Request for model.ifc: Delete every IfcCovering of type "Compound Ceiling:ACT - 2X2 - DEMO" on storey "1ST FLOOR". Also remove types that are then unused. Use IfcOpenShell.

First a look at what the model holds.

```python
import ifcopenshell
import ifcopenshell.util.element

model = ifcopenshell.open("model.ifc")
print(model.schema)
storey = next(s for s in model.by_type("IfcBuildingStorey") if s.Name == "1ST FLOOR")
coverings = [e for e in ifcopenshell.util.element.get_decomposition(storey) if e.is_a("IfcCovering")]
seen = {}
for e in coverings:
    element_type = ifcopenshell.util.element.get_type(e)
    name = element_type.Name if element_type not in (None, e) else None
    seen[name] = seen.get(name, 0) + 1
for name, count in sorted(seen.items(), key=str):
    print(count, "x", name)
```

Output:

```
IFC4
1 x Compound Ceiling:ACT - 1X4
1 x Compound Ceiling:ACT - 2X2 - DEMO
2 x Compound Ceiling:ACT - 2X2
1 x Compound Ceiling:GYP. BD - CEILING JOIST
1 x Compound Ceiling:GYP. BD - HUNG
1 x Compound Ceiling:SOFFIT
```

```python
import ifcopenshell
import ifcopenshell.api.root
import ifcopenshell.util.element

model = ifcopenshell.open("model.ifc")

storey = next(s for s in model.by_type("IfcBuildingStorey") if s.Name == "1ST FLOOR")
coverings = [e for e in ifcopenshell.util.element.get_decomposition(storey) if e.is_a("IfcCovering")]
targets = [e for e in coverings if (t := ifcopenshell.util.element.get_type(e)) not in (None, e) and t.Name == "Compound Ceiling:ACT - 2X2 - DEMO"]
types = {ifcopenshell.util.element.get_type(e) for e in targets} - {None, *targets}

for e in targets:
    ifcopenshell.api.root.remove_product(model, product=e)
print(len(targets), "removed")

unused = [t for t in types if not ifcopenshell.util.element.get_types(t)]
for t in unused:
    ifcopenshell.api.root.remove_product(model, product=t)
print(len(unused), "unused types removed")

model.write("model_v2.ifc")
```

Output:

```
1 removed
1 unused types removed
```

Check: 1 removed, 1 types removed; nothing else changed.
